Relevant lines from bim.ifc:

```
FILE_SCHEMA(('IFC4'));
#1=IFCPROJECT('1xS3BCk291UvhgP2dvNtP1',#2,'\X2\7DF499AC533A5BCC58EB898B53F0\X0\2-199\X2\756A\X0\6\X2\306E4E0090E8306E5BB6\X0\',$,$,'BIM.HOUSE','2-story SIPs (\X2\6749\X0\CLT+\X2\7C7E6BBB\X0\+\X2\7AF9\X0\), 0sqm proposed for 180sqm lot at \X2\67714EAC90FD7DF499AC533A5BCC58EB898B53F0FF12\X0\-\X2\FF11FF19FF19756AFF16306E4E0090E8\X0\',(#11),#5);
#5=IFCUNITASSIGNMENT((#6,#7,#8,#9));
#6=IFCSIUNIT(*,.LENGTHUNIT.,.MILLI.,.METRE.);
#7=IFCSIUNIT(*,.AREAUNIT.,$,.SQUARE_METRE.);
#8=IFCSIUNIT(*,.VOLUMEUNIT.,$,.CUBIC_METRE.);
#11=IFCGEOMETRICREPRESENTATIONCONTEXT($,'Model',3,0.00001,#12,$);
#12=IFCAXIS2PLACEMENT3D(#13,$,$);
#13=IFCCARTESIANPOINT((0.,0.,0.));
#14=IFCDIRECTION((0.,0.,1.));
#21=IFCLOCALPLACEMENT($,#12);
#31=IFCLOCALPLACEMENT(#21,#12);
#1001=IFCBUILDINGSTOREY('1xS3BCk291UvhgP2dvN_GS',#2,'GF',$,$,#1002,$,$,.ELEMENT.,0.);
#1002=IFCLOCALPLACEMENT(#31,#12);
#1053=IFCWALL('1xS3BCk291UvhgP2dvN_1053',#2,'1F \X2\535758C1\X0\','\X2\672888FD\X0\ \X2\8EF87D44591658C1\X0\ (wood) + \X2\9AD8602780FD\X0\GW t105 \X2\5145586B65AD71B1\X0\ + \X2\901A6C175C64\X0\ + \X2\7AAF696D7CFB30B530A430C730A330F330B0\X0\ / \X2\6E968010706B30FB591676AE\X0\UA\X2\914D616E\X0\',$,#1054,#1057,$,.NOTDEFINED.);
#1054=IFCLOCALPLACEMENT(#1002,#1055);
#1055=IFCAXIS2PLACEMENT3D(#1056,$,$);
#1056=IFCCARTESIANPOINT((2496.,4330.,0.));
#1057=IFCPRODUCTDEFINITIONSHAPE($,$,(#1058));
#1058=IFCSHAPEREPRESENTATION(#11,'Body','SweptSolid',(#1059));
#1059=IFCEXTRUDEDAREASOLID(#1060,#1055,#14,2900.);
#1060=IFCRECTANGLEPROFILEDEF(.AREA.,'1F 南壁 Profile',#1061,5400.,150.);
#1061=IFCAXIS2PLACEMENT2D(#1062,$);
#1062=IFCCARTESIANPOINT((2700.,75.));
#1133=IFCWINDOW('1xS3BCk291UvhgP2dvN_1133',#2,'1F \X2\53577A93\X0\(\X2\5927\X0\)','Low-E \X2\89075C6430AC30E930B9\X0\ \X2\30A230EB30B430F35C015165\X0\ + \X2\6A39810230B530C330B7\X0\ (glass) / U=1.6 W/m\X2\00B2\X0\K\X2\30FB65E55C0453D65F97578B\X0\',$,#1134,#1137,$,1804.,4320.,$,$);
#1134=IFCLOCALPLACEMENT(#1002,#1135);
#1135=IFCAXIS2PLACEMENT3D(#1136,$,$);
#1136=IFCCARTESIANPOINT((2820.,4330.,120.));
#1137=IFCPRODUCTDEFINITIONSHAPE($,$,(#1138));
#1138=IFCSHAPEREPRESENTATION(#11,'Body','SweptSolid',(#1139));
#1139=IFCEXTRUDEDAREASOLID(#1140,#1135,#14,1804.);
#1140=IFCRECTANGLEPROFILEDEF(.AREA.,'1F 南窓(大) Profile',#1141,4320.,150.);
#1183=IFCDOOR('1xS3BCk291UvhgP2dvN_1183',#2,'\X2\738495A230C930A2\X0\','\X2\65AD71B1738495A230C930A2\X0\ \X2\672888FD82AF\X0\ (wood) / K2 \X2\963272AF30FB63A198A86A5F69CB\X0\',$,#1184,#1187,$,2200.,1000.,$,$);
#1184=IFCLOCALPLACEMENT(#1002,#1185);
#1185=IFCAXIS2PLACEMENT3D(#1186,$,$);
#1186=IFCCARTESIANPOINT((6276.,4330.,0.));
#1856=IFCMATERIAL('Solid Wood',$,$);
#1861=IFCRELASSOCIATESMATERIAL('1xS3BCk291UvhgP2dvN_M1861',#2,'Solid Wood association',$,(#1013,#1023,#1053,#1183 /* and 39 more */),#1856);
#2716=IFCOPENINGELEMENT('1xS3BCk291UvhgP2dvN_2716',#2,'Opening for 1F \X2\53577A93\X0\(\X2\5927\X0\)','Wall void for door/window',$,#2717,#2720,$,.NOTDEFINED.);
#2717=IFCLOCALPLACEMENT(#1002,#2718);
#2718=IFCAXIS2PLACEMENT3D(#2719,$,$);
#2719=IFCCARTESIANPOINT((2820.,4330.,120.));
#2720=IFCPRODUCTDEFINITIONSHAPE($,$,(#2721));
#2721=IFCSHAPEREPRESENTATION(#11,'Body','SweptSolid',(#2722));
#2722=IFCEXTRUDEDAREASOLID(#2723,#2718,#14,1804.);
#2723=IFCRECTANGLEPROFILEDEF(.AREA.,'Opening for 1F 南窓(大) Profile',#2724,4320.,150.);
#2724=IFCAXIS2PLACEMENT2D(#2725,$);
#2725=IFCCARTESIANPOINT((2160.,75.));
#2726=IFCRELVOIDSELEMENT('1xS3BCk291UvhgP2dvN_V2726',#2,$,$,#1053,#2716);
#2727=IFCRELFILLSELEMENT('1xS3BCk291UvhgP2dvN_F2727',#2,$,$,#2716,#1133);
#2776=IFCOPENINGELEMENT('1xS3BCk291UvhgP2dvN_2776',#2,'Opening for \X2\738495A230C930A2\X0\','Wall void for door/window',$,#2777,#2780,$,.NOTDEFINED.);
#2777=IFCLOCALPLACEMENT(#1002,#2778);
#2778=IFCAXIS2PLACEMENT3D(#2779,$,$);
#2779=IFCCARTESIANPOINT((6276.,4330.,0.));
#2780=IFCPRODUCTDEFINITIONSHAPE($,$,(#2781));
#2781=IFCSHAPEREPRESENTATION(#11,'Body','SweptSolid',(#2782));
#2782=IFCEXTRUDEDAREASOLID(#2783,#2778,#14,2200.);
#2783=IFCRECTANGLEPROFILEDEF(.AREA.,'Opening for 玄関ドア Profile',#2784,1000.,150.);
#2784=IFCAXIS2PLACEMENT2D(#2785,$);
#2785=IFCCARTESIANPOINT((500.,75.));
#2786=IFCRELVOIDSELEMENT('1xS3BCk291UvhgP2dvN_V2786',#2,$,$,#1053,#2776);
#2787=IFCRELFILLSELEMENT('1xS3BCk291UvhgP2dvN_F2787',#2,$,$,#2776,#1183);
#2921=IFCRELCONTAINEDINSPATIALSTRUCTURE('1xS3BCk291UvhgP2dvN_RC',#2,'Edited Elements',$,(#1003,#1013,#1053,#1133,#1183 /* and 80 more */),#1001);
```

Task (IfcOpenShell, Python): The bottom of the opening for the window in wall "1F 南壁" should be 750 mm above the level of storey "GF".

```python
import numpy as np
import ifcopenshell
import ifcopenshell.api.geometry
import ifcopenshell.geom
import ifcopenshell.util.element
import ifcopenshell.util.placement
import ifcopenshell.util.shape
import ifcopenshell.util.unit

model = ifcopenshell.open("bim.ifc")
unit_scale = ifcopenshell.util.unit.calculate_unit_scale(model)

window = model.by_guid("1xS3BCk291UvhgP2dvN_1133")
opening = window.FillsVoids[0].RelatingOpeningElement
storey = ifcopenshell.util.element.get_container(window, ifc_class="IfcBuildingStorey")
level = ifcopenshell.util.placement.get_local_placement(storey.ObjectPlacement)[2, 3]

# The opening's origin need not be at the sill, so measure its lowest point.
shape = ifcopenshell.geom.create_shape(ifcopenshell.geom.settings(), opening)
bottom = ifcopenshell.util.shape.get_shape_bottom_elevation(shape, shape.geometry) / unit_scale
dz = level + 0.75 / unit_scale - bottom

shift = np.array([0.0, 0.0, dz])
# The window is not placed relative to its opening, so move both.
for product in (opening, window):
    matrix = ifcopenshell.util.placement.get_local_placement(product.ObjectPlacement)
    matrix[:3, 3] += shift
    ifcopenshell.api.geometry.edit_object_placement(model, product=product, matrix=matrix, is_si=False)

print(f"moved by {dz * unit_scale:+.3f} m")

model.write("bim_updated.ifc")
```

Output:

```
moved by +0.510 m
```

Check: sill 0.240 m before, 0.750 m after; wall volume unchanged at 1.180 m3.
